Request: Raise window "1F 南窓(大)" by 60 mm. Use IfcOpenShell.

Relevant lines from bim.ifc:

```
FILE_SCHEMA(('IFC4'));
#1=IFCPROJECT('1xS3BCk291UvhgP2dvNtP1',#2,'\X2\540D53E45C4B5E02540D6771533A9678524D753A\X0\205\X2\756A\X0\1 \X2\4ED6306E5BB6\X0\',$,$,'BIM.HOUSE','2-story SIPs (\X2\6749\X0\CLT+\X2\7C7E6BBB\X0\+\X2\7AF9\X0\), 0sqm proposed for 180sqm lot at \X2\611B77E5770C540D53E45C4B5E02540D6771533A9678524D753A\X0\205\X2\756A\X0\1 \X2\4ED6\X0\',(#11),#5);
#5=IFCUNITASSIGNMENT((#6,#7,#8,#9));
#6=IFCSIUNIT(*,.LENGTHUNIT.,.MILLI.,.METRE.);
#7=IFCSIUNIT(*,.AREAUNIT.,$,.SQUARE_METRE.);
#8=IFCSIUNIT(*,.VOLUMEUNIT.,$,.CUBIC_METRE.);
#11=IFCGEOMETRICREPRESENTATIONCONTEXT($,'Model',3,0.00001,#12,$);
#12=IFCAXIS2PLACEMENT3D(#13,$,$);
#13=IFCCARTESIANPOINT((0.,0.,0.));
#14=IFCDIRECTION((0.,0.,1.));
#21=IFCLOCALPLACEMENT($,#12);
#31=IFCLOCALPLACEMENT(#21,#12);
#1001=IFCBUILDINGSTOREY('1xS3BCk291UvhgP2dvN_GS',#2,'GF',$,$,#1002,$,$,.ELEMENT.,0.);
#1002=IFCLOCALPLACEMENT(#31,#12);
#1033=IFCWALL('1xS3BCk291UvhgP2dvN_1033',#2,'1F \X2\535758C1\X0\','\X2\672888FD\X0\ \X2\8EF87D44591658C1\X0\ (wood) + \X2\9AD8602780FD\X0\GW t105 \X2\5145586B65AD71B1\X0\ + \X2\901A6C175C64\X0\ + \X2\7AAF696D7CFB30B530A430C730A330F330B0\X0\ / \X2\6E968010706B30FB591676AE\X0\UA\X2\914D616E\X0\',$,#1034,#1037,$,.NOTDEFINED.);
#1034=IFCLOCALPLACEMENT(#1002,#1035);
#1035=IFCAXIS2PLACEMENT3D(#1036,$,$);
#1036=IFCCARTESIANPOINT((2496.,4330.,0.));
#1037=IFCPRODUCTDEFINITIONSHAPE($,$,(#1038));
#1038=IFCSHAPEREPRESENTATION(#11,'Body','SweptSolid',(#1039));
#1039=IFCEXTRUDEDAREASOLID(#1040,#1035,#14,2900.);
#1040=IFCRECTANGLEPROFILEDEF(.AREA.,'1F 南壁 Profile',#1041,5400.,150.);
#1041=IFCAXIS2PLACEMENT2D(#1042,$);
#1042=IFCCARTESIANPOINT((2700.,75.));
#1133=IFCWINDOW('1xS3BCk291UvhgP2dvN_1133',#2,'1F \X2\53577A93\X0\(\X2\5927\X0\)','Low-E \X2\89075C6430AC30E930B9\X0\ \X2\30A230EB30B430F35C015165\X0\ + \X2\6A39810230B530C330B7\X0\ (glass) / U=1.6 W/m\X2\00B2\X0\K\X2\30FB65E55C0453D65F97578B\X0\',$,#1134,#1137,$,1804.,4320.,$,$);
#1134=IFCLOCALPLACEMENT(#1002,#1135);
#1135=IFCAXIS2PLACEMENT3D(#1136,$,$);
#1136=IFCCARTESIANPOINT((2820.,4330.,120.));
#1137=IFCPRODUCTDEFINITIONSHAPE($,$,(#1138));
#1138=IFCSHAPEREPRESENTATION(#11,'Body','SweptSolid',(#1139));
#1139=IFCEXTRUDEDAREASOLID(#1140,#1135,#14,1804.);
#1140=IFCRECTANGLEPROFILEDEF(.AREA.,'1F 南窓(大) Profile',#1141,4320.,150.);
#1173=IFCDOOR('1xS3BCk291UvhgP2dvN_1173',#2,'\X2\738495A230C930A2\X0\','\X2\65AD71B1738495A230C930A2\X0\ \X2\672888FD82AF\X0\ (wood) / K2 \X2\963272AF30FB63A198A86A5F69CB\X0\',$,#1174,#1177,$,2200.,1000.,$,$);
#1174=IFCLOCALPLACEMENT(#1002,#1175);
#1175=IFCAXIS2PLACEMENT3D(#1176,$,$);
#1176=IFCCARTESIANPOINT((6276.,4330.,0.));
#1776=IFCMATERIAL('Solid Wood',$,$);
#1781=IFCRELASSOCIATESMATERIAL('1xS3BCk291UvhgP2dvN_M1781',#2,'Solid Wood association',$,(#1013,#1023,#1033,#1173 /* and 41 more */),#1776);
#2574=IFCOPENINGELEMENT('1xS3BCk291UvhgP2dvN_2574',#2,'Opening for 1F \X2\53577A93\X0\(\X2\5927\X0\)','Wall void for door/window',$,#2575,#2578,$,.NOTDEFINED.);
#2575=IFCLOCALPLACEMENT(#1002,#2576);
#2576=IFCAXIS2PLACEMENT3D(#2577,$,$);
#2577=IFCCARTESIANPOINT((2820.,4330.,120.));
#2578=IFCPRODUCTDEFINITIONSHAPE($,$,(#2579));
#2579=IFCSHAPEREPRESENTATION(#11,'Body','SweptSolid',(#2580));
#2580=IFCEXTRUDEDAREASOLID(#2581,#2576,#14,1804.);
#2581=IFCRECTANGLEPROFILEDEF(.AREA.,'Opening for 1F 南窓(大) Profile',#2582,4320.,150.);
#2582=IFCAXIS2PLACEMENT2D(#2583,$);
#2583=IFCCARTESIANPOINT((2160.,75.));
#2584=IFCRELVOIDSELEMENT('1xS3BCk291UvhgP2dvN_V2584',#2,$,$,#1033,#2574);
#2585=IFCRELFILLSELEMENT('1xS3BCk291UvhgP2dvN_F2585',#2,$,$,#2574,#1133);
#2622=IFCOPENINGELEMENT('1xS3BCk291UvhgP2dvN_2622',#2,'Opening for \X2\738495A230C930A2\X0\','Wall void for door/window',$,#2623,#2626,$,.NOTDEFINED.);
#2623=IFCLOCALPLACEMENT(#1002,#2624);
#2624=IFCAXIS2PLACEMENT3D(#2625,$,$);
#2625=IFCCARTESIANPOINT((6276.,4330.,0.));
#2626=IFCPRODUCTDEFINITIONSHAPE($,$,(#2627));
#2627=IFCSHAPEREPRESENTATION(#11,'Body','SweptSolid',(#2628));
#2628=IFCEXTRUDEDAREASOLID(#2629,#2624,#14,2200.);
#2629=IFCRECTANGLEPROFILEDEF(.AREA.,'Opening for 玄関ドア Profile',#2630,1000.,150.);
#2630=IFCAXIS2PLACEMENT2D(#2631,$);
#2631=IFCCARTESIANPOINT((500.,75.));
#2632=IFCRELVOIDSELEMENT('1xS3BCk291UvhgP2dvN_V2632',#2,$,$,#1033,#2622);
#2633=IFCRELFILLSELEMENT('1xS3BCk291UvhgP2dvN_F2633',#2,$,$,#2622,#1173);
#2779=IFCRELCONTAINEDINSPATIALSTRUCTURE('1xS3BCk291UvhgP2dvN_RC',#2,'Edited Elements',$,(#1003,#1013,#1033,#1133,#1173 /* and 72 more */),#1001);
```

```python
import numpy as np
import ifcopenshell
import ifcopenshell.api.geometry
import ifcopenshell.util.placement
import ifcopenshell.util.unit

model = ifcopenshell.open("bim.ifc")
unit_scale = ifcopenshell.util.unit.calculate_unit_scale(model)

window = model.by_id(1133)
opening = window.FillsVoids[0].RelatingOpeningElement
dz = 0.06 / unit_scale

shift = np.array([0.0, 0.0, dz])
# The window is not placed relative to its opening, so move both.
for product in (opening, window):
    matrix = ifcopenshell.util.placement.get_local_placement(product.ObjectPlacement)
    matrix[:3, 3] += shift
    ifcopenshell.api.geometry.edit_object_placement(model, product=product, matrix=matrix, is_si=False)

print(f"moved by {dz * unit_scale:+.3f} m")

model.write("bim-out.ifc")
```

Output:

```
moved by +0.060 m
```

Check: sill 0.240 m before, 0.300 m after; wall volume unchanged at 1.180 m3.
